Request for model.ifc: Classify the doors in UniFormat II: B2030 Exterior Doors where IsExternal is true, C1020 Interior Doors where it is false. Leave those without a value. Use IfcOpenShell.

First a look at what the model holds.

```python
import ifcopenshell
import ifcopenshell.util.element

model = ifcopenshell.open("model.ifc")
print(model.schema)
print("classifications:", [c.Name for c in model.by_type("IfcClassification")])
values = [ifcopenshell.util.element.get_pset(e, "Pset_DoorCommon", "IsExternal") for e in model.by_type("IfcDoor")]
for value in (True, False, None):
    print("IsExternal", value, values.count(value))
```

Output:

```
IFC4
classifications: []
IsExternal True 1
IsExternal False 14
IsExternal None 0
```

```python
import ifcopenshell
import ifcopenshell.api.classification
import ifcopenshell.util.element

model = ifcopenshell.open("model.ifc")

system = ifcopenshell.api.classification.add_classification(model, classification="UniFormat II")

doors = model.by_type("IfcDoor")
external = {e: ifcopenshell.util.element.get_pset(e, "Pset_DoorCommon", "IsExternal") for e in doors}
for flag, code, name in ((True, "B2030", "Exterior Doors"), (False, "C1020", "Interior Doors")):
    products = [e for e in doors if external[e] is flag]
    ifcopenshell.api.classification.add_reference(
        model, products=products, classification=system, identification=code, name=name
    )
    print(code, len(products))

model.write("model_updated.ifc")
```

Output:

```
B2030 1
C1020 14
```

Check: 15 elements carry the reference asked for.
